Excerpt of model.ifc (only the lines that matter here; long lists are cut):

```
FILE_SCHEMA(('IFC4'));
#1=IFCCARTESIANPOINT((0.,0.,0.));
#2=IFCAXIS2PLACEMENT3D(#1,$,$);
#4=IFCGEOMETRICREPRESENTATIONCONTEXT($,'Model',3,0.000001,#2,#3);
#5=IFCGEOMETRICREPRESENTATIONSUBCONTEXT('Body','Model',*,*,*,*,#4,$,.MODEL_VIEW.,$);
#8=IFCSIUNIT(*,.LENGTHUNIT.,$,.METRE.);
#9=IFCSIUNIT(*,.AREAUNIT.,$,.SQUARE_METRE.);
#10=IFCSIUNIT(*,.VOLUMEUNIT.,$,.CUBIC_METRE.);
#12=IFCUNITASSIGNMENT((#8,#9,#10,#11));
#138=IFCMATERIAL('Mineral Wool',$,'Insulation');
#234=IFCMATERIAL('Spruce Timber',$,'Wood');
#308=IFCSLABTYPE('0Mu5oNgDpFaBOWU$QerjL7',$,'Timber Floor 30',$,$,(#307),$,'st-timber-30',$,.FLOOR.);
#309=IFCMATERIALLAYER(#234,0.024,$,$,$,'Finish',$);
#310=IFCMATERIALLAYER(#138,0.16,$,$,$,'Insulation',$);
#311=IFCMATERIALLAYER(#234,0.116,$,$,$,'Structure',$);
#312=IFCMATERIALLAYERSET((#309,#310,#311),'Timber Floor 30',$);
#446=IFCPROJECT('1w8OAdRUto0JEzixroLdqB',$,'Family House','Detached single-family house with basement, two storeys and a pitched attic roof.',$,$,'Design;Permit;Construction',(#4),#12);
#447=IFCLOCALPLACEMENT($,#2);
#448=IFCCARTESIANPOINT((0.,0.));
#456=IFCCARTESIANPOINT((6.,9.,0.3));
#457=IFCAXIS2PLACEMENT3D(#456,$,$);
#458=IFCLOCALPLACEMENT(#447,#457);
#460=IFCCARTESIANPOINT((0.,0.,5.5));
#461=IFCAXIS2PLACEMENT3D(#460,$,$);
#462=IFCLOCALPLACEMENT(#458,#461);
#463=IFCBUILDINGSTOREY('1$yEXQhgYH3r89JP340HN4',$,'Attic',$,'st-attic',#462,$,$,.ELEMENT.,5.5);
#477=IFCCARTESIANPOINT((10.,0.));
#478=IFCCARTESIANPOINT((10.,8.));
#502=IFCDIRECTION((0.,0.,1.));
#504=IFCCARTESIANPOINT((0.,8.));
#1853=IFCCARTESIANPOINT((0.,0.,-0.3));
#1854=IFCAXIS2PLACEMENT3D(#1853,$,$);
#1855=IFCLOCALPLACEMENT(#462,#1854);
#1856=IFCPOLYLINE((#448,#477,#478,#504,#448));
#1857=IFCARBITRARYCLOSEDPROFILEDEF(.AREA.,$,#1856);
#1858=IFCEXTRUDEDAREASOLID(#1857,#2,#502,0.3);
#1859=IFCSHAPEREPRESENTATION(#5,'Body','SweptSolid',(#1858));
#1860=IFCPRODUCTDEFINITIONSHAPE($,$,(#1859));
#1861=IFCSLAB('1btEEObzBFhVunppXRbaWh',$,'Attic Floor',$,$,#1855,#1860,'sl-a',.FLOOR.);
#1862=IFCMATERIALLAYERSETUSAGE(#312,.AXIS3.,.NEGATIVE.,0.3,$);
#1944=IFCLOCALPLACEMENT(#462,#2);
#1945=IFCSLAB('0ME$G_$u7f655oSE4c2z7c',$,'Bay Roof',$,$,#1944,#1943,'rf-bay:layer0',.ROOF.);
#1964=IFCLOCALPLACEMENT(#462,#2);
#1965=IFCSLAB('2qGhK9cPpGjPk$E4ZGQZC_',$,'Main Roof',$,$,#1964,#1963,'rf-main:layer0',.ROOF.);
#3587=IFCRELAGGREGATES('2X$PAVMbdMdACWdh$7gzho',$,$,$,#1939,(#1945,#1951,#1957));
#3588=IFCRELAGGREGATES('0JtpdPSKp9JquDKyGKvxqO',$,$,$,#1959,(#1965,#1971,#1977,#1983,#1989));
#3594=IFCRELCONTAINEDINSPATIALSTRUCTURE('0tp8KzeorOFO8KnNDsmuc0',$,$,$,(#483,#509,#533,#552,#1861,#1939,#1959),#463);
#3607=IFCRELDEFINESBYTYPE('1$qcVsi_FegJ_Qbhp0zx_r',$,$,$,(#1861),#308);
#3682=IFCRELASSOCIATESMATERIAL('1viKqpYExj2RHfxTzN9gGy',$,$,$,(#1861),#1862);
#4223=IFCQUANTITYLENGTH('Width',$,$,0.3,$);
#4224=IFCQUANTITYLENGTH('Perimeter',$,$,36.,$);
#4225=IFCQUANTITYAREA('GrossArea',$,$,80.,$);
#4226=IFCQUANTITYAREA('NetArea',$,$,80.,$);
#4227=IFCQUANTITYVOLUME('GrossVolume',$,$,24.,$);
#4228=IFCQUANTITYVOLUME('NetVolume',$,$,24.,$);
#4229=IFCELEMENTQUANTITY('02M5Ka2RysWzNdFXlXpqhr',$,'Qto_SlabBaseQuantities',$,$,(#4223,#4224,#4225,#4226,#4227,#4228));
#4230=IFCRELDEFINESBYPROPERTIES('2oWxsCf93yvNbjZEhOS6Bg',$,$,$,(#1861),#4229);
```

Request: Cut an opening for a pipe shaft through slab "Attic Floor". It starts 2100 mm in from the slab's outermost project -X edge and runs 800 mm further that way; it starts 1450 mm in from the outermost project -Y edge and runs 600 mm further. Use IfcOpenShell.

```python
import numpy as np
import ifcopenshell
import ifcopenshell.api.feature
import ifcopenshell.api.geometry
import ifcopenshell.api.pset
import ifcopenshell.api.root
import ifcopenshell.geom
import ifcopenshell.util.element
import ifcopenshell.util.placement
import ifcopenshell.util.representation
import ifcopenshell.util.shape
import ifcopenshell.util.unit

model = ifcopenshell.open("model.ifc")
unit_scale = ifcopenshell.util.unit.calculate_unit_scale(model)
area_scale = ifcopenshell.util.unit.calculate_unit_scale(model, "AREAUNIT")
volume_scale = ifcopenshell.util.unit.calculate_unit_scale(model, "VOLUMEUNIT")
settings = ifcopenshell.geom.settings()


def volume(element):
    """Net volume in cubic metres, openings subtracted."""
    shape = ifcopenshell.geom.create_shape(settings, element)
    return ifcopenshell.util.shape.get_volume(shape.geometry)


slab = model.by_guid("1btEEObzBFhVunppXRbaWh")
before = volume(slab)

# Extent in the slab's own axes, in metres. The edges named are its -X and -Y sides.
slab_shape = ifcopenshell.geom.create_shape(settings, slab)
vertices = ifcopenshell.util.shape.get_vertices(slab_shape.geometry)
x_min, y_min, bottom = vertices.min(axis=0)
top = vertices[:, 2].max()

opening = ifcopenshell.api.root.create_entity(model, ifc_class="IfcOpeningElement", name="Pipe shaft opening", predefined_type="OPENING")
context = ifcopenshell.util.representation.get_context(model, "Model", "Body", "MODEL_VIEW")
width, depth = 0.8, 0.6
outline = [(0.0, 0.0), (width, 0.0), (width, depth), (0.0, depth), (0.0, 0.0)]
# Overshoot both faces by 50 mm so the cut is clean.
shape = ifcopenshell.api.geometry.add_slab_representation(
    model, context=context, depth=top - bottom + 0.1, polyline=outline
)
ifcopenshell.api.geometry.assign_representation(model, product=opening, representation=shape)

matrix = ifcopenshell.util.placement.get_local_placement(slab.ObjectPlacement)
matrix[:, 3] = matrix @ np.append(np.array([x_min + 2.1, y_min + 1.45, bottom - 0.05]) / unit_scale, 1.0)
ifcopenshell.api.geometry.edit_object_placement(model, product=opening, matrix=matrix, is_si=False)
ifcopenshell.api.feature.add_feature(model, feature=opening, element=slab)

after = volume(slab)

# Update the slab's stored quantities.
qto = model.by_id(ifcopenshell.util.element.get_pset(slab, "Qto_SlabBaseQuantities", should_inherit=False)["id"])
ifcopenshell.api.pset.edit_qto(model, qto=qto, properties={
    "NetArea": after / (top - bottom) / area_scale,
    "NetVolume": after / volume_scale,
})

print(f"slab volume {before:.3f} -> {after:.3f} m3")

model.write("model_v2.ifc")
```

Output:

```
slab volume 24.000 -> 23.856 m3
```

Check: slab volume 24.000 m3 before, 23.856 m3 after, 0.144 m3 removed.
